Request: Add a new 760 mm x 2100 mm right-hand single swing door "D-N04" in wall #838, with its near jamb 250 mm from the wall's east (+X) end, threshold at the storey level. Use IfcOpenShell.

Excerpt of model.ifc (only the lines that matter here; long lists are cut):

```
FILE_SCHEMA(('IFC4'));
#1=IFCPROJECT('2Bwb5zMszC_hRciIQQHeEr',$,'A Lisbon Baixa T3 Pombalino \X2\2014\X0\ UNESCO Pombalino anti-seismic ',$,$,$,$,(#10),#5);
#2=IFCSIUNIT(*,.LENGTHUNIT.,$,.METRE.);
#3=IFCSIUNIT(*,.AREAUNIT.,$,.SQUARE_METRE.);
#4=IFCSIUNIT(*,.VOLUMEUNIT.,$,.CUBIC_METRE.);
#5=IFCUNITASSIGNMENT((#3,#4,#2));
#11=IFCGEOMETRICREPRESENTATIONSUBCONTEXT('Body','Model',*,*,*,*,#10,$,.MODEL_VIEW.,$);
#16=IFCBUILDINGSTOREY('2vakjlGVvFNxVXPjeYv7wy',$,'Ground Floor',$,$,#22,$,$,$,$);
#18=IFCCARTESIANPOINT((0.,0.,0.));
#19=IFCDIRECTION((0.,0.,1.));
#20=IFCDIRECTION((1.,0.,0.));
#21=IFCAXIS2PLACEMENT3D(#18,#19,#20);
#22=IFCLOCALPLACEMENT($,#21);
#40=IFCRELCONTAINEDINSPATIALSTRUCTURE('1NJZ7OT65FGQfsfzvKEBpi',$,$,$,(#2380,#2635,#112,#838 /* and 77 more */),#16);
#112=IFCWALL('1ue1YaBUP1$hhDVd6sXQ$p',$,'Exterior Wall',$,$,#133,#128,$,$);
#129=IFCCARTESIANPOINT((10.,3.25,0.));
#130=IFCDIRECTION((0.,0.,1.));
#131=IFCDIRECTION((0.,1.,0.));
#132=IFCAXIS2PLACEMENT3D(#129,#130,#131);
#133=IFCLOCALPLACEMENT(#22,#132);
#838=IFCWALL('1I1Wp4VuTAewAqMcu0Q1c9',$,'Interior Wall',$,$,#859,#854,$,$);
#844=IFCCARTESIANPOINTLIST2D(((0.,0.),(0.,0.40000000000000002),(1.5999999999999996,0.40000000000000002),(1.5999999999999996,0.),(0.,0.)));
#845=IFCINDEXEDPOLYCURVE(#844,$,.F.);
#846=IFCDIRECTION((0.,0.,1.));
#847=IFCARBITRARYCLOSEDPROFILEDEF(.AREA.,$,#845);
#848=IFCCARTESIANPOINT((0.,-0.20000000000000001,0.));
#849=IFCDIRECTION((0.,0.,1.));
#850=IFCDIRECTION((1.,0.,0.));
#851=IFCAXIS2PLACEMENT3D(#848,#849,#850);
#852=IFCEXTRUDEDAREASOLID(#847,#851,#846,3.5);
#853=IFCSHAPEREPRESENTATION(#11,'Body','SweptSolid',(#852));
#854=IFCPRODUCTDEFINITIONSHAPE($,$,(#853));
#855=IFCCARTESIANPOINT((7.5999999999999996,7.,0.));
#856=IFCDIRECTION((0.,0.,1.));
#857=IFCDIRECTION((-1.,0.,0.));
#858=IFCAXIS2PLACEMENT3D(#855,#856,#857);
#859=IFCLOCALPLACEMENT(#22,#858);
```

```python
import numpy as np
import ifcopenshell
import ifcopenshell.api.feature
import ifcopenshell.api.geometry
import ifcopenshell.api.root
import ifcopenshell.api.spatial
import ifcopenshell.geom
import ifcopenshell.util.element
import ifcopenshell.util.placement
import ifcopenshell.util.representation
import ifcopenshell.util.shape
import ifcopenshell.util.unit

model = ifcopenshell.open("model.ifc")
unit_scale = ifcopenshell.util.unit.calculate_unit_scale(model)
settings = ifcopenshell.geom.settings()


def volume(element):
    """Net volume in cubic metres, openings subtracted."""
    shape = ifcopenshell.geom.create_shape(settings, element)
    return ifcopenshell.util.shape.get_volume(shape.geometry)


wall = model.by_guid("1I1Wp4VuTAewAqMcu0Q1c9")
storey = ifcopenshell.util.element.get_container(wall, ifc_class="IfcBuildingStorey")
context = ifcopenshell.util.representation.get_context(model, "Model", "Body", "MODEL_VIEW")
before = volume(wall)

width, height, from_end, sill = 0.76, 2.1, 0.25, 0.0  # metres

# The wall runs along its own X axis, and the end named is its -X end.
wall_shape = ifcopenshell.geom.create_shape(settings, wall)
x, y, z = ifcopenshell.util.shape.get_vertices(wall_shape.geometry).T
start = x.min() + from_end
face, thickness = float(y.min()), float(y.max() - y.min())
wall_matrix = ifcopenshell.util.placement.get_local_placement(wall.ObjectPlacement)
level = ifcopenshell.util.placement.get_local_placement(storey.ObjectPlacement)[2, 3]


def in_wall(x, y):
    """Placement at x, y metres in the wall's axes, at sill height."""
    matrix = wall_matrix.copy()
    matrix[:, 3] = wall_matrix @ np.array([x / unit_scale, y / unit_scale, 0.0, 1.0])
    matrix[2, 3] = level + sill / unit_scale
    return matrix


# Opening: a box that overshoots both wall faces by 50 mm.
opening = ifcopenshell.api.root.create_entity(model, ifc_class="IfcOpeningElement", predefined_type="OPENING")
box = ifcopenshell.api.geometry.add_wall_representation(
    model, context=context, length=width, height=height, thickness=thickness + 0.1
)
ifcopenshell.api.geometry.assign_representation(model, product=opening, representation=box)
ifcopenshell.api.geometry.edit_object_placement(model, product=opening, matrix=in_wall(start, face - 0.05), is_si=False)
ifcopenshell.api.feature.add_feature(model, feature=opening, element=wall)

door = ifcopenshell.api.root.create_entity(model, ifc_class="IfcDoor", name="D-N04", predefined_type="DOOR")
door.OverallWidth, door.OverallHeight = width / unit_scale, height / unit_scale
door.OperationType = "SINGLE_SWING_RIGHT"
body = ifcopenshell.api.geometry.add_door_representation(
    model,
    context=context,
    overall_width=door.OverallWidth,
    overall_height=door.OverallHeight,
    operation_type="SINGLE_SWING_RIGHT",
    lining_properties={"LiningDepth": thickness / unit_scale, "ThresholdDepth": thickness / unit_scale},
)
ifcopenshell.api.geometry.assign_representation(model, product=door, representation=body)
ifcopenshell.api.spatial.assign_container(model, products=[door], relating_structure=storey)
ifcopenshell.api.feature.add_filling(model, opening=opening, element=door)

# The lining spans the wall, so the door starts at the wall face.
ifcopenshell.api.geometry.edit_object_placement(model, product=door, matrix=in_wall(start, face), is_si=False)

after = volume(wall)

print(f"wall volume {before:.3f} -> {after:.3f} m3")

model.write("model_updated.ifc")
```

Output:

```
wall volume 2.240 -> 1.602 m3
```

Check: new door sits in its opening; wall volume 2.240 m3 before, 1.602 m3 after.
